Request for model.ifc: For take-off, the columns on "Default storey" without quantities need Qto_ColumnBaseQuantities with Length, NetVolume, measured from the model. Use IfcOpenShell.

First a look at what the model holds.

```python
import ifcopenshell
import ifcopenshell.util.element
import ifcopenshell.util.unit

model = ifcopenshell.open("model.ifc")
print(model.schema)
for unit_type in ("LENGTHUNIT", "AREAUNIT", "VOLUMEUNIT"):
    print(unit_type, ifcopenshell.util.unit.calculate_unit_scale(model, unit_type))
storey = next(s for s in model.by_type("IfcBuildingStorey") if s.Name == "Default storey")
columns = [e for e in ifcopenshell.util.element.get_decomposition(storey) if e.is_a("IfcColumn")]
for e in sorted(columns, key=lambda e: e.id()):
    print(e.id(), e.is_a(), e.Name, list(ifcopenshell.util.element.get_psets(e, qtos_only=True)), sep=" | ")
```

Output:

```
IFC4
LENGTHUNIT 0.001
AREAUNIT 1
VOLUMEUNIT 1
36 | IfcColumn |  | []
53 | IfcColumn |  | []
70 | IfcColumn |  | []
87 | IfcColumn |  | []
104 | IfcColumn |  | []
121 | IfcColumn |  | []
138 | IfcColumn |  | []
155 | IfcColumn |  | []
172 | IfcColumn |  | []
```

```python
import ifcopenshell
import ifcopenshell.api.pset
import ifcopenshell.geom
import ifcopenshell.util.element
import ifcopenshell.util.shape
import ifcopenshell.util.unit

model = ifcopenshell.open("model.ifc")
unit_scale = ifcopenshell.util.unit.calculate_unit_scale(model)
volume_scale = ifcopenshell.util.unit.calculate_unit_scale(model, "VOLUMEUNIT")
settings = ifcopenshell.geom.settings()

storey = next(s for s in model.by_type("IfcBuildingStorey") if s.Name == "Default storey")
columns = [e for e in ifcopenshell.util.element.get_decomposition(storey) if e.is_a("IfcColumn")]

for e in sorted(columns, key=lambda e: e.id()):
    if ifcopenshell.util.element.get_psets(e, qtos_only=True, should_inherit=False):
        continue
    # Geometry comes back in metres, in the element's own axes.
    shape = ifcopenshell.geom.create_shape(settings, e)
    values = {
        "Length": ifcopenshell.util.shape.get_z(shape.geometry) / unit_scale,
        "NetVolume": ifcopenshell.util.shape.get_volume(shape.geometry) / volume_scale,
    }
    qto = ifcopenshell.api.pset.add_qto(model, product=e, name="Qto_ColumnBaseQuantities")
    ifcopenshell.api.pset.edit_qto(model, qto=qto, properties=values)
    print(e.id(), {k: round(v, 3) for k, v in values.items()})

model.write("model_rev.ifc")
```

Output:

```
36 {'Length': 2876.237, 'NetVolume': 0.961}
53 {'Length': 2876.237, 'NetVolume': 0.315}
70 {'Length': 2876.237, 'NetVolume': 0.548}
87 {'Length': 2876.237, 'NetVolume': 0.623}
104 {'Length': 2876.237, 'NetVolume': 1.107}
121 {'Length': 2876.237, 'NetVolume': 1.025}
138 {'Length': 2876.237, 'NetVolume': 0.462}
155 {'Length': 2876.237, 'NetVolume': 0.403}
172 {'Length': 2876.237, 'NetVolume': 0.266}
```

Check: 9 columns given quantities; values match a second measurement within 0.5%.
